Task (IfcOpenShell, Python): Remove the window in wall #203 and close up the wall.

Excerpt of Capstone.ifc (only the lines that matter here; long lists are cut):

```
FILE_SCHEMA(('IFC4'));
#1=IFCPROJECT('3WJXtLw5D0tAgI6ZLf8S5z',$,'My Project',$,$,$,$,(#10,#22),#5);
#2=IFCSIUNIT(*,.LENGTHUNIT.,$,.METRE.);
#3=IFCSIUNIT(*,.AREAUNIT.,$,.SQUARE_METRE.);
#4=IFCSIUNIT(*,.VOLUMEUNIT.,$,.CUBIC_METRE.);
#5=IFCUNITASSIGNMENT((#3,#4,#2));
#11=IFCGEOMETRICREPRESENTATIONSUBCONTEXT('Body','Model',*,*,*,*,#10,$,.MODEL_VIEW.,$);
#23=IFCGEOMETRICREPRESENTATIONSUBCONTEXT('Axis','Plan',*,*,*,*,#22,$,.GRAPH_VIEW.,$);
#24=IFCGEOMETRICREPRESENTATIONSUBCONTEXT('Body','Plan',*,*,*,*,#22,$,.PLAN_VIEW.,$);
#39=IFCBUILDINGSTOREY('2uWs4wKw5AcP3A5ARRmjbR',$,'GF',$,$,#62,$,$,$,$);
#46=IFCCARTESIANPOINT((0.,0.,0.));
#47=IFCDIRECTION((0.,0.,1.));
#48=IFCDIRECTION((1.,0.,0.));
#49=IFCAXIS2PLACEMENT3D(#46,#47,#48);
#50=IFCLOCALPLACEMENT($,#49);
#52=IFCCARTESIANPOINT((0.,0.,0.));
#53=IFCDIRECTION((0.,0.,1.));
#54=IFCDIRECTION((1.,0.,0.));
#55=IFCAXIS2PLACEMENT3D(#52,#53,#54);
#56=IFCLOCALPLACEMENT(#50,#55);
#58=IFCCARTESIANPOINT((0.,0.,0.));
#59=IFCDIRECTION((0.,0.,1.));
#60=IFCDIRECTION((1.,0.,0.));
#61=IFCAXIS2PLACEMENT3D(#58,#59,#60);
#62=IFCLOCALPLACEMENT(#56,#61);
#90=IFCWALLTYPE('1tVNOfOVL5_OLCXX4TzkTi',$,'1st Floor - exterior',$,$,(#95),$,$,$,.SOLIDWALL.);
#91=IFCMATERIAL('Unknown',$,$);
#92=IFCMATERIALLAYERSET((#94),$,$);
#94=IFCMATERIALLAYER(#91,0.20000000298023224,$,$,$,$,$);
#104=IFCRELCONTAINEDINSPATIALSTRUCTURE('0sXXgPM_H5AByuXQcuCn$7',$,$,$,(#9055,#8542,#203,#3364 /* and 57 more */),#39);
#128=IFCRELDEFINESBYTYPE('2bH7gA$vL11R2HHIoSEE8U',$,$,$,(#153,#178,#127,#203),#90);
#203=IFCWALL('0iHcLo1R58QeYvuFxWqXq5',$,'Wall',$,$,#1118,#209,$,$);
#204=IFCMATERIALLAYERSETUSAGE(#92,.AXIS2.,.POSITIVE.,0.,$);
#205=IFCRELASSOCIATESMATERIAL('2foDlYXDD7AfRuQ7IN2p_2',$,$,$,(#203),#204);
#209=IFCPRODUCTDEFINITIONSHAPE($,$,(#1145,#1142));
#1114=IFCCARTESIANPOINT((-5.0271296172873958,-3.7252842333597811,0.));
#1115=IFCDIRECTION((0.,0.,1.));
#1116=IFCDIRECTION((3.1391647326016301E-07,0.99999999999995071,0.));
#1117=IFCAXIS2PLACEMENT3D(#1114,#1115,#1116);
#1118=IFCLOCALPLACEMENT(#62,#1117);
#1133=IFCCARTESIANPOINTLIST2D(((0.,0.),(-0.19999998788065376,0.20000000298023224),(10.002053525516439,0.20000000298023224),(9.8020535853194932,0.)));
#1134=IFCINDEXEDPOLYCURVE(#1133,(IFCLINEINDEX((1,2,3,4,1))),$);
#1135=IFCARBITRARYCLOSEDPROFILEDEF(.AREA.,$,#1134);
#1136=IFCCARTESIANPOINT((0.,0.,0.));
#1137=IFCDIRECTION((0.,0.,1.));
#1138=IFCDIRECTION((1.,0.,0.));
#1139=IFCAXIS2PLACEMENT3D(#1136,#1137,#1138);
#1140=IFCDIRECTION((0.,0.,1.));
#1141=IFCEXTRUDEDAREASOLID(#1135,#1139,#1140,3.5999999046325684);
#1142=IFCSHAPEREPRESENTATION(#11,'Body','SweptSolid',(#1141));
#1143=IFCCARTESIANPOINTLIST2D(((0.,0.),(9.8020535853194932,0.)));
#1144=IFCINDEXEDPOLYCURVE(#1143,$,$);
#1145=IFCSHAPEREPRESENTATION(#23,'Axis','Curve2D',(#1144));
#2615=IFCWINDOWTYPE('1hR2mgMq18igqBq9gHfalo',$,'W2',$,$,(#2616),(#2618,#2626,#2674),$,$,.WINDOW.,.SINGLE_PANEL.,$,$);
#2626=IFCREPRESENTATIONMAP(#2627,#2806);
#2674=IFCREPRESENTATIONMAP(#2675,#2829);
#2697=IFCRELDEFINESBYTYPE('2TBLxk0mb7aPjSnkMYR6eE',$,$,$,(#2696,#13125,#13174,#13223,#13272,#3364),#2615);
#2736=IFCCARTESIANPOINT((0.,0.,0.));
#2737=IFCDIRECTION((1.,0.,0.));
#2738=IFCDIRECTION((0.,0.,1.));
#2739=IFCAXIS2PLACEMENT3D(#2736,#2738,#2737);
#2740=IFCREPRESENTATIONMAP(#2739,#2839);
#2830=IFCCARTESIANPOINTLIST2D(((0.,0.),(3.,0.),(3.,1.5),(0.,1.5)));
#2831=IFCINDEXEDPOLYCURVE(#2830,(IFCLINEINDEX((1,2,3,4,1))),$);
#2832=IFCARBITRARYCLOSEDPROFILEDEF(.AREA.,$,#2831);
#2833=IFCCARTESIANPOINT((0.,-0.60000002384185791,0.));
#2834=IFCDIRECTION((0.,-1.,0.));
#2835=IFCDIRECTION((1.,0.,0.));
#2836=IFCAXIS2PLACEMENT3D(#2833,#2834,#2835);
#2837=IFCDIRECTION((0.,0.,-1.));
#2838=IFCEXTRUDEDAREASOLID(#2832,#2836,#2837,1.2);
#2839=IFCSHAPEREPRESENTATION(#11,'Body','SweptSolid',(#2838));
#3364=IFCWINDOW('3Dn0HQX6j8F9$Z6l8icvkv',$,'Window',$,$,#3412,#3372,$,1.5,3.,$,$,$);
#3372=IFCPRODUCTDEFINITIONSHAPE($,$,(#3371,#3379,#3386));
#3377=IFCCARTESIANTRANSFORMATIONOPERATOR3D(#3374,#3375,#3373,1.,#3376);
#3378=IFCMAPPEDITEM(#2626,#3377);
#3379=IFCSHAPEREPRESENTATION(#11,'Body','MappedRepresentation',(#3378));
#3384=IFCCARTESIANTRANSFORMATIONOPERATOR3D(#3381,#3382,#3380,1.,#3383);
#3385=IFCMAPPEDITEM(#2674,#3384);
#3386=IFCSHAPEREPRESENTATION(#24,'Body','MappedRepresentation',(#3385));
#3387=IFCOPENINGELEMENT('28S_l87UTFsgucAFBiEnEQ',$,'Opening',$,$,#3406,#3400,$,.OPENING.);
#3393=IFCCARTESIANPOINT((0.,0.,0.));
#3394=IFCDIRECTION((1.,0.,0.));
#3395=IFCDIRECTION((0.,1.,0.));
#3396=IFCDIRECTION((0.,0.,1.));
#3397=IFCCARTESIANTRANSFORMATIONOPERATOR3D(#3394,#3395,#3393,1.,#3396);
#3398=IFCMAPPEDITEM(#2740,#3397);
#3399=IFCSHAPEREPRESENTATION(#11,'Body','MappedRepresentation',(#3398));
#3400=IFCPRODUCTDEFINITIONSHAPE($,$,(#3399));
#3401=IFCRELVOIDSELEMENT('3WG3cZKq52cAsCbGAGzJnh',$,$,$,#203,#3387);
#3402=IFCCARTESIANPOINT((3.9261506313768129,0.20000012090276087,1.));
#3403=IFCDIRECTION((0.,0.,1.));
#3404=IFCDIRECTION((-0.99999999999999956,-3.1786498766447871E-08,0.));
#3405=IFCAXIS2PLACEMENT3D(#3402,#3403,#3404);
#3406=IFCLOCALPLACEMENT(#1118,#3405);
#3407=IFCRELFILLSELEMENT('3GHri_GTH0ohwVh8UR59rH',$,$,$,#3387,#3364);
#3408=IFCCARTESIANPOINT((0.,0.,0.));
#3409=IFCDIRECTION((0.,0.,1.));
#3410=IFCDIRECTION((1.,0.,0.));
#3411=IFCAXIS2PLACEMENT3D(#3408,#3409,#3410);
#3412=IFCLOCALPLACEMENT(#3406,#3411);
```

```python
import ifcopenshell
import ifcopenshell.api.feature
import ifcopenshell.api.root
import ifcopenshell.geom
import ifcopenshell.util.shape

model = ifcopenshell.open("Capstone.ifc")
settings = ifcopenshell.geom.settings()


def volume(element):
    """Net volume in cubic metres, openings subtracted."""
    shape = ifcopenshell.geom.create_shape(settings, element)
    return ifcopenshell.util.shape.get_volume(shape.geometry)


window = model.by_guid("3Dn0HQX6j8F9$Z6l8icvkv")
opening = window.FillsVoids[0].RelatingOpeningElement
wall = opening.VoidsElements[0].RelatingBuildingElement
before = volume(wall)

ifcopenshell.api.root.remove_product(model, product=window)
ifcopenshell.api.feature.remove_feature(model, feature=opening)

after = volume(wall)

print(f"wall volume {before:.3f} -> {after:.3f} m3")

model.write("Capstone_v2.ifc")
```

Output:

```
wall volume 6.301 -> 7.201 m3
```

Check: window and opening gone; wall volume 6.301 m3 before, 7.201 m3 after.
